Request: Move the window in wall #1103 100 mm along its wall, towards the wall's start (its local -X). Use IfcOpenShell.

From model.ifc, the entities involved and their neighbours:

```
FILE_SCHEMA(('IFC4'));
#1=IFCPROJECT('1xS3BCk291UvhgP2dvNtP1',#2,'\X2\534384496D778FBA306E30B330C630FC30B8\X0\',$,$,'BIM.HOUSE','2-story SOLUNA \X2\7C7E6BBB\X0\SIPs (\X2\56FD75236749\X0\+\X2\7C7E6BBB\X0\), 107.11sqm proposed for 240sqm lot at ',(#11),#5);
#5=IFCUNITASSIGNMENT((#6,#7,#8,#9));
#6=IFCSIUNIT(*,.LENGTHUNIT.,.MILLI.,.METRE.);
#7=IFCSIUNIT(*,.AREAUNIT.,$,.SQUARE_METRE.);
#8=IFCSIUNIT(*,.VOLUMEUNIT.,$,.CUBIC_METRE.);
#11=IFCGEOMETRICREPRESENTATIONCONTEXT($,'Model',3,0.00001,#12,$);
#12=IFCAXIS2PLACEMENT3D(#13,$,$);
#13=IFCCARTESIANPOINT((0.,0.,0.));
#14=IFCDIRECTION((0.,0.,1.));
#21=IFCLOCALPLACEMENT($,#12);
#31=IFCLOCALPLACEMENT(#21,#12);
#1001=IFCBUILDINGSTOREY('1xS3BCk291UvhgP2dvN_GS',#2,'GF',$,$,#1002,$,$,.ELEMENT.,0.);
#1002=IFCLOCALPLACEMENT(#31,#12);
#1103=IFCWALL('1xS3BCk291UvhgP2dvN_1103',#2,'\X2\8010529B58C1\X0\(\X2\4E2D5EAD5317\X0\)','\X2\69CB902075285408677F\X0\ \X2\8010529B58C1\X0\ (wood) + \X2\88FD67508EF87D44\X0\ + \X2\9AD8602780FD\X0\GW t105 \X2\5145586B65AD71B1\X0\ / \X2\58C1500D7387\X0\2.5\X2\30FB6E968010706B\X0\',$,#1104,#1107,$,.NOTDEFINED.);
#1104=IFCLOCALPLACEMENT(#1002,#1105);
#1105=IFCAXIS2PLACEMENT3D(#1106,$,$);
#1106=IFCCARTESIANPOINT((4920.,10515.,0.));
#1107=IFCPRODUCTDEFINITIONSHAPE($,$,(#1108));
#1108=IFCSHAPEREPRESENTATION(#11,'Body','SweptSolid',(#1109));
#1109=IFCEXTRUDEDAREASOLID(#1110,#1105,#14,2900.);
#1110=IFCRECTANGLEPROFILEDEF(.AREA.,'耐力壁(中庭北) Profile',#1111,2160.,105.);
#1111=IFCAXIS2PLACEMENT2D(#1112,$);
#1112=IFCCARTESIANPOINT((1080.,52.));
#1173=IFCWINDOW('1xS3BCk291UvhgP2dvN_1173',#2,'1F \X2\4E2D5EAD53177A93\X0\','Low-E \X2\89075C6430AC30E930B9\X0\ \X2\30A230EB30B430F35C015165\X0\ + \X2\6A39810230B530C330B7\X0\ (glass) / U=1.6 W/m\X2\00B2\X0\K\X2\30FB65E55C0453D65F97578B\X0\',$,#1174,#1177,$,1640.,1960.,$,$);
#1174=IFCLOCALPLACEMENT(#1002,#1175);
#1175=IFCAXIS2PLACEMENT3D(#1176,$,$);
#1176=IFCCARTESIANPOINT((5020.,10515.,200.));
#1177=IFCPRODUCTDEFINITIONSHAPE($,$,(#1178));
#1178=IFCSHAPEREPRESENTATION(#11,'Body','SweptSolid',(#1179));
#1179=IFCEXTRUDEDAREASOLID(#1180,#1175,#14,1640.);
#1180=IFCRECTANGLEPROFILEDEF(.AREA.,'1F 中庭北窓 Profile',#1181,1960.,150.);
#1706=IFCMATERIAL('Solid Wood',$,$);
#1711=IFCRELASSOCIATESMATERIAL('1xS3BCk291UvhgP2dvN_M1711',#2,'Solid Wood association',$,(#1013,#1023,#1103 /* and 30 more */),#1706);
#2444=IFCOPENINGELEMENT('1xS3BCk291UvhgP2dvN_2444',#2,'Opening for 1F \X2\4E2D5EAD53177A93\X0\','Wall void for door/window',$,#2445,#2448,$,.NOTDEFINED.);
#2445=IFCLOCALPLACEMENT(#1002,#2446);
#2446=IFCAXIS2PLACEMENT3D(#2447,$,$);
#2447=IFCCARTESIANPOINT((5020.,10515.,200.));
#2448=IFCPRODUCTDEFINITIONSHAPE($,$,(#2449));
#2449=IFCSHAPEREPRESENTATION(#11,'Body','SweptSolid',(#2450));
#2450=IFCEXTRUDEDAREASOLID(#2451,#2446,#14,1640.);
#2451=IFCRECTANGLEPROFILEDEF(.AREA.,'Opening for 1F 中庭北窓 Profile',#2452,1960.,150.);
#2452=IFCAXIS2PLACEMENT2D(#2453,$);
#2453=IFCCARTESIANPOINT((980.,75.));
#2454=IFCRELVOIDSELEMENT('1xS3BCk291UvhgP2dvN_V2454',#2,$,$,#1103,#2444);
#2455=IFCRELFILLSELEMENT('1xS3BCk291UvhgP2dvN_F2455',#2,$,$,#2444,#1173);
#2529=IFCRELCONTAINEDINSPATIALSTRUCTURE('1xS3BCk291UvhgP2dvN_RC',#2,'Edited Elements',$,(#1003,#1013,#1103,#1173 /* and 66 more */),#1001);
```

```python
import ifcopenshell
import ifcopenshell.api.geometry
import ifcopenshell.util.placement
import ifcopenshell.util.unit

model = ifcopenshell.open("model.ifc")
unit_scale = ifcopenshell.util.unit.calculate_unit_scale(model)

window = model.by_guid("1xS3BCk291UvhgP2dvN_1173")
opening = window.FillsVoids[0].RelatingOpeningElement
wall = opening.VoidsElements[0].RelatingBuildingElement

wall_matrix = ifcopenshell.util.placement.get_local_placement(wall.ObjectPlacement)
shift = wall_matrix[:3, 0] * -0.1 / unit_scale
before = ifcopenshell.util.placement.get_local_placement(window.ObjectPlacement)[:3, 3].copy()

# The window is not placed relative to its opening, so move both.
for product in (opening, window):
    matrix = ifcopenshell.util.placement.get_local_placement(product.ObjectPlacement)
    matrix[:3, 3] += shift
    ifcopenshell.api.geometry.edit_object_placement(model, product=product, matrix=matrix, is_si=False)

after = ifcopenshell.util.placement.get_local_placement(window.ObjectPlacement)[:3, 3]
print("window moved by", (after - before).round(3) + 0.0)

model.write("model_rev.ifc")
```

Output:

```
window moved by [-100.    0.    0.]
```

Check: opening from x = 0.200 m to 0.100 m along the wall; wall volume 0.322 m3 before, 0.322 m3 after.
